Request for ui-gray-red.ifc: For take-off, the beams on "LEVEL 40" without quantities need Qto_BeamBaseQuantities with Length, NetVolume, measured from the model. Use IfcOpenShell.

First a look at what the model holds.

```python
import ifcopenshell
import ifcopenshell.util.element
import ifcopenshell.util.unit

model = ifcopenshell.open("ui-gray-red.ifc")
print(model.schema)
for unit_type in ("LENGTHUNIT", "AREAUNIT", "VOLUMEUNIT"):
    print(unit_type, ifcopenshell.util.unit.calculate_unit_scale(model, unit_type))
storey = next(s for s in model.by_type("IfcBuildingStorey") if s.Name == "LEVEL 40")
beams = [e for e in ifcopenshell.util.element.get_decomposition(storey) if e.is_a("IfcBeam")]
for e in sorted(beams, key=lambda e: e.id()):
    print(e.id(), e.is_a(), e.Name, list(ifcopenshell.util.element.get_psets(e, qtos_only=True)), sep=" | ")
```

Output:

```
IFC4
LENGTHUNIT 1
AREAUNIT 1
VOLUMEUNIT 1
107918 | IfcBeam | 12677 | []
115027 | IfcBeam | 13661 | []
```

```python
import ifcopenshell
import ifcopenshell.api.pset
import ifcopenshell.geom
import ifcopenshell.util.element
import ifcopenshell.util.shape
import ifcopenshell.util.unit

model = ifcopenshell.open("ui-gray-red.ifc")
unit_scale = ifcopenshell.util.unit.calculate_unit_scale(model)
volume_scale = ifcopenshell.util.unit.calculate_unit_scale(model, "VOLUMEUNIT")
settings = ifcopenshell.geom.settings()

storey = next(s for s in model.by_type("IfcBuildingStorey") if s.Name == "LEVEL 40")
beams = [e for e in ifcopenshell.util.element.get_decomposition(storey) if e.is_a("IfcBeam")]

for e in sorted(beams, key=lambda e: e.id()):
    if ifcopenshell.util.element.get_psets(e, qtos_only=True, should_inherit=False):
        continue
    # Geometry comes back in metres, in the element's own axes.
    shape = ifcopenshell.geom.create_shape(settings, e)
    values = {
        "Length": ifcopenshell.util.shape.get_max_xyz(shape.geometry) / unit_scale,
        "NetVolume": ifcopenshell.util.shape.get_volume(shape.geometry) / volume_scale,
    }
    qto = ifcopenshell.api.pset.add_qto(model, product=e, name="Qto_BeamBaseQuantities")
    ifcopenshell.api.pset.edit_qto(model, qto=qto, properties=values)
    print(e.id(), {k: round(v, 3) for k, v in values.items()})

model.write("ui-gray-red_edited.ifc")
```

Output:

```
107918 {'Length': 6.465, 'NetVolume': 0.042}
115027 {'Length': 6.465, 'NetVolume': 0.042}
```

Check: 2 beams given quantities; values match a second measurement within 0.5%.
